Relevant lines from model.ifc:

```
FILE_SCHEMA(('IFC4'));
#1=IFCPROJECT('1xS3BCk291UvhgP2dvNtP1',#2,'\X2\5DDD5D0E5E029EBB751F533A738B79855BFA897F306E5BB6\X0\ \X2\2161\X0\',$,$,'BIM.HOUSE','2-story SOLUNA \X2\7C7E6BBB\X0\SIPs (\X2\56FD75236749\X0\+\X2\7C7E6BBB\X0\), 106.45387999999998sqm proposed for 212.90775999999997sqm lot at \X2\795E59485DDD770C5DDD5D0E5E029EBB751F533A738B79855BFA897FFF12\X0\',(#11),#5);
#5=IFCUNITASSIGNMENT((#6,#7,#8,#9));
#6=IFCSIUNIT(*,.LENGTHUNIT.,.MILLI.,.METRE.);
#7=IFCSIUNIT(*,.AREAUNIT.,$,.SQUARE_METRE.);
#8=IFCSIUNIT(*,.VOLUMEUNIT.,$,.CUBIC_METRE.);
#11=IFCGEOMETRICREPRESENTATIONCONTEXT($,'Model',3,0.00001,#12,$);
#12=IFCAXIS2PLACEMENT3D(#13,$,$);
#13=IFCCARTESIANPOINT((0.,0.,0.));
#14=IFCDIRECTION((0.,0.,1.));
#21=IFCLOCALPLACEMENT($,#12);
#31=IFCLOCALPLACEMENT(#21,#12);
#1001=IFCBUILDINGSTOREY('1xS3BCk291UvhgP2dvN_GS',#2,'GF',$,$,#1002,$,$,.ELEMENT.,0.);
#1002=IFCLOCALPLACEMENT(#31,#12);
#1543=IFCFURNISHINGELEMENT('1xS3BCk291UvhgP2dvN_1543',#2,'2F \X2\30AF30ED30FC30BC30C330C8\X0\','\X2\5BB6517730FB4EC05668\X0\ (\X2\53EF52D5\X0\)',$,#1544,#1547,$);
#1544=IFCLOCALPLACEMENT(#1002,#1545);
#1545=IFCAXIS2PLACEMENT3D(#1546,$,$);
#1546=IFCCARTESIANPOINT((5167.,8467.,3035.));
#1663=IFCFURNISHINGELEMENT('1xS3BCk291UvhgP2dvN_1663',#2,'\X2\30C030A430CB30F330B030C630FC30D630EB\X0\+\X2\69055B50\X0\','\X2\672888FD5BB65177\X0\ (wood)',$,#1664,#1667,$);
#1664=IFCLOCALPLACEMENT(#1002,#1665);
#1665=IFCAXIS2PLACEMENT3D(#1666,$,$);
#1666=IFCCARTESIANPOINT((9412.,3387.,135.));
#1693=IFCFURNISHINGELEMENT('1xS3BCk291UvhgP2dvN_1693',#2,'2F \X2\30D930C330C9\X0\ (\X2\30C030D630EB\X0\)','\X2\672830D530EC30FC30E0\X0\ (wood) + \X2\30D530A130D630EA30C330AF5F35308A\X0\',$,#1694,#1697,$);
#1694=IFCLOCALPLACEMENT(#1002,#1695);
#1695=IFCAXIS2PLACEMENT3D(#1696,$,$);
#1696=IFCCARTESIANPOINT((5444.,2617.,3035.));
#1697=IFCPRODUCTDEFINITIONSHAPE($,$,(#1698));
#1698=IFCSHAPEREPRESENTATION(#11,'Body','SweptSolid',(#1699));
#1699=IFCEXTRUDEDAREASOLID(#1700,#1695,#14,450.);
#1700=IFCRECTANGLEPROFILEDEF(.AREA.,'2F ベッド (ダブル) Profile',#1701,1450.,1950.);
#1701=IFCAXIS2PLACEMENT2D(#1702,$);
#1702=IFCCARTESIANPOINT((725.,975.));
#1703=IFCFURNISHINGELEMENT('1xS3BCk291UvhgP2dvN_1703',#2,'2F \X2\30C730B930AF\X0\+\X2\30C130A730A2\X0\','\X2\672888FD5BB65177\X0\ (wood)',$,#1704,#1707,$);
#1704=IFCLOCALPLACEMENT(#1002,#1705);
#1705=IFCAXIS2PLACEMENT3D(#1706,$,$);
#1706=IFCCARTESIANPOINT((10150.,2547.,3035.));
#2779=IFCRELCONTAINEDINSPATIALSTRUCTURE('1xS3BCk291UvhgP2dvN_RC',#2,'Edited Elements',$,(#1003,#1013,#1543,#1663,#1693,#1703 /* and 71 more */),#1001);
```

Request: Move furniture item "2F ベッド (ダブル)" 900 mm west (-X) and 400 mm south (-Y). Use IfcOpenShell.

```python
import ifcopenshell
import ifcopenshell.api.geometry
import ifcopenshell.util.placement
import ifcopenshell.util.unit

model = ifcopenshell.open("model.ifc")
unit_scale = ifcopenshell.util.unit.calculate_unit_scale(model)

item = model.by_guid("1xS3BCk291UvhgP2dvN_1693")
matrix = ifcopenshell.util.placement.get_local_placement(item.ObjectPlacement)
matrix[0, 3] -= 0.9 / unit_scale
matrix[1, 3] -= 0.4 / unit_scale
ifcopenshell.api.geometry.edit_object_placement(model, product=item, matrix=matrix, is_si=False)

print(ifcopenshell.util.placement.get_local_placement(item.ObjectPlacement).round(3) + 0.0)

model.write("model_edited.ifc")
```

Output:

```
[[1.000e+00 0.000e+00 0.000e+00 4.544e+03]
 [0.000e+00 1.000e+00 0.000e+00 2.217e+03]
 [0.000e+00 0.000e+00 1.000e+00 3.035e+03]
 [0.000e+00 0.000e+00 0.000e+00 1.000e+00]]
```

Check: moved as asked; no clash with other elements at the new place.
